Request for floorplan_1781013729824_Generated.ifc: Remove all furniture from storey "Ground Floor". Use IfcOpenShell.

First a look at what the model holds.

```python
import ifcopenshell
import ifcopenshell.util.element

model = ifcopenshell.open("floorplan_1781013729824_Generated.ifc")
print(model.schema)
storey = next(s for s in model.by_type("IfcBuildingStorey") if s.Name == "Ground Floor")
furniture = [e for e in ifcopenshell.util.element.get_decomposition(storey) if e.is_a("IfcFurnishingElement")]
seen = {}
for e in furniture:
    element_type = ifcopenshell.util.element.get_type(e)
    name = element_type.Name if element_type not in (None, e) else None
    seen[name] = seen.get(name, 0) + 1
for name, count in sorted(seen.items(), key=str):
    print(count, "x", name)
```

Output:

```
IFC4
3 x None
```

```python
import ifcopenshell
import ifcopenshell.api.root
import ifcopenshell.util.element

model = ifcopenshell.open("floorplan_1781013729824_Generated.ifc")

storey = next(s for s in model.by_type("IfcBuildingStorey") if s.Name == "Ground Floor")
furniture = [e for e in ifcopenshell.util.element.get_decomposition(storey) if e.is_a("IfcFurnishingElement")]

for e in furniture:
    ifcopenshell.api.root.remove_product(model, product=e)
print(len(furniture), "removed")

model.write("floorplan_1781013729824_Generated_rev.ifc")
```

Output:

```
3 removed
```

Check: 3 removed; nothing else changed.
